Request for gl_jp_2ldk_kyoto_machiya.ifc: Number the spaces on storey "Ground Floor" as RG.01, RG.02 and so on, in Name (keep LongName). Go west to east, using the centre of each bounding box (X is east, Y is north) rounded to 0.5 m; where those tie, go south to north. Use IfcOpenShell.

First a look at what the model holds.

```python
import ifcopenshell
import ifcopenshell.util.element
import ifcopenshell.util.placement

model = ifcopenshell.open("gl_jp_2ldk_kyoto_machiya.ifc")
print(model.schema)
storey = next(s for s in model.by_type("IfcBuildingStorey") if s.Name == "Ground Floor")
spaces = [e for e in ifcopenshell.util.element.get_decomposition(storey) if e.is_a("IfcSpace")]
for e in sorted(spaces, key=lambda e: e.id()):
    origin = ifcopenshell.util.placement.get_local_placement(e.ObjectPlacement)[:3, 3]
    print(e.id(), e.Name, e.LongName, origin.round(2) + 0.0, sep=" | ")
```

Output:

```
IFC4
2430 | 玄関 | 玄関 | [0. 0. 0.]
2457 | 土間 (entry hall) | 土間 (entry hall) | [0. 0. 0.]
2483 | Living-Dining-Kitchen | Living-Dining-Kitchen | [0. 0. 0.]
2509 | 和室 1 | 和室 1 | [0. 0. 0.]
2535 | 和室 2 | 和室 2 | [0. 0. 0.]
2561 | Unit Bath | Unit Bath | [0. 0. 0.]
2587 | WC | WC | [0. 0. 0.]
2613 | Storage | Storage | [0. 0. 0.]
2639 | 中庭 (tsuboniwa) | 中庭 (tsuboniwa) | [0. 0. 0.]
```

```python
import ifcopenshell
import ifcopenshell.geom
import ifcopenshell.util.element
import ifcopenshell.util.shape

model = ifcopenshell.open("gl_jp_2ldk_kyoto_machiya.ifc")
settings = ifcopenshell.geom.settings()
settings.set("use-world-coords", True)


def centre(element):
    shape = ifcopenshell.geom.create_shape(settings, element)
    return ifcopenshell.util.shape.get_bbox_centroid(shape.geometry)


storey = next(s for s in model.by_type("IfcBuildingStorey") if s.Name == "Ground Floor")
spaces = [e for e in ifcopenshell.util.element.get_decomposition(storey) if e.is_a("IfcSpace")]

# Insertion points can sit at a corner or the storey origin, so sort by the geometry (in metres).
centres = {e: centre(e) for e in spaces}
spaces.sort(key=lambda e: (round(centres[e][0] / 0.5), centres[e][1]))

for i, e in enumerate(spaces, start=1):
    number = f"RG.{i:02d}"
    e.Name = number
    print(e.id(), number)

model.write("gl_jp_2ldk_kyoto_machiya_rev.ifc")
```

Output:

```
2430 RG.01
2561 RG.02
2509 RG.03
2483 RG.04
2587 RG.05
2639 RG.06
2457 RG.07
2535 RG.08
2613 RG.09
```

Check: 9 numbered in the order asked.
